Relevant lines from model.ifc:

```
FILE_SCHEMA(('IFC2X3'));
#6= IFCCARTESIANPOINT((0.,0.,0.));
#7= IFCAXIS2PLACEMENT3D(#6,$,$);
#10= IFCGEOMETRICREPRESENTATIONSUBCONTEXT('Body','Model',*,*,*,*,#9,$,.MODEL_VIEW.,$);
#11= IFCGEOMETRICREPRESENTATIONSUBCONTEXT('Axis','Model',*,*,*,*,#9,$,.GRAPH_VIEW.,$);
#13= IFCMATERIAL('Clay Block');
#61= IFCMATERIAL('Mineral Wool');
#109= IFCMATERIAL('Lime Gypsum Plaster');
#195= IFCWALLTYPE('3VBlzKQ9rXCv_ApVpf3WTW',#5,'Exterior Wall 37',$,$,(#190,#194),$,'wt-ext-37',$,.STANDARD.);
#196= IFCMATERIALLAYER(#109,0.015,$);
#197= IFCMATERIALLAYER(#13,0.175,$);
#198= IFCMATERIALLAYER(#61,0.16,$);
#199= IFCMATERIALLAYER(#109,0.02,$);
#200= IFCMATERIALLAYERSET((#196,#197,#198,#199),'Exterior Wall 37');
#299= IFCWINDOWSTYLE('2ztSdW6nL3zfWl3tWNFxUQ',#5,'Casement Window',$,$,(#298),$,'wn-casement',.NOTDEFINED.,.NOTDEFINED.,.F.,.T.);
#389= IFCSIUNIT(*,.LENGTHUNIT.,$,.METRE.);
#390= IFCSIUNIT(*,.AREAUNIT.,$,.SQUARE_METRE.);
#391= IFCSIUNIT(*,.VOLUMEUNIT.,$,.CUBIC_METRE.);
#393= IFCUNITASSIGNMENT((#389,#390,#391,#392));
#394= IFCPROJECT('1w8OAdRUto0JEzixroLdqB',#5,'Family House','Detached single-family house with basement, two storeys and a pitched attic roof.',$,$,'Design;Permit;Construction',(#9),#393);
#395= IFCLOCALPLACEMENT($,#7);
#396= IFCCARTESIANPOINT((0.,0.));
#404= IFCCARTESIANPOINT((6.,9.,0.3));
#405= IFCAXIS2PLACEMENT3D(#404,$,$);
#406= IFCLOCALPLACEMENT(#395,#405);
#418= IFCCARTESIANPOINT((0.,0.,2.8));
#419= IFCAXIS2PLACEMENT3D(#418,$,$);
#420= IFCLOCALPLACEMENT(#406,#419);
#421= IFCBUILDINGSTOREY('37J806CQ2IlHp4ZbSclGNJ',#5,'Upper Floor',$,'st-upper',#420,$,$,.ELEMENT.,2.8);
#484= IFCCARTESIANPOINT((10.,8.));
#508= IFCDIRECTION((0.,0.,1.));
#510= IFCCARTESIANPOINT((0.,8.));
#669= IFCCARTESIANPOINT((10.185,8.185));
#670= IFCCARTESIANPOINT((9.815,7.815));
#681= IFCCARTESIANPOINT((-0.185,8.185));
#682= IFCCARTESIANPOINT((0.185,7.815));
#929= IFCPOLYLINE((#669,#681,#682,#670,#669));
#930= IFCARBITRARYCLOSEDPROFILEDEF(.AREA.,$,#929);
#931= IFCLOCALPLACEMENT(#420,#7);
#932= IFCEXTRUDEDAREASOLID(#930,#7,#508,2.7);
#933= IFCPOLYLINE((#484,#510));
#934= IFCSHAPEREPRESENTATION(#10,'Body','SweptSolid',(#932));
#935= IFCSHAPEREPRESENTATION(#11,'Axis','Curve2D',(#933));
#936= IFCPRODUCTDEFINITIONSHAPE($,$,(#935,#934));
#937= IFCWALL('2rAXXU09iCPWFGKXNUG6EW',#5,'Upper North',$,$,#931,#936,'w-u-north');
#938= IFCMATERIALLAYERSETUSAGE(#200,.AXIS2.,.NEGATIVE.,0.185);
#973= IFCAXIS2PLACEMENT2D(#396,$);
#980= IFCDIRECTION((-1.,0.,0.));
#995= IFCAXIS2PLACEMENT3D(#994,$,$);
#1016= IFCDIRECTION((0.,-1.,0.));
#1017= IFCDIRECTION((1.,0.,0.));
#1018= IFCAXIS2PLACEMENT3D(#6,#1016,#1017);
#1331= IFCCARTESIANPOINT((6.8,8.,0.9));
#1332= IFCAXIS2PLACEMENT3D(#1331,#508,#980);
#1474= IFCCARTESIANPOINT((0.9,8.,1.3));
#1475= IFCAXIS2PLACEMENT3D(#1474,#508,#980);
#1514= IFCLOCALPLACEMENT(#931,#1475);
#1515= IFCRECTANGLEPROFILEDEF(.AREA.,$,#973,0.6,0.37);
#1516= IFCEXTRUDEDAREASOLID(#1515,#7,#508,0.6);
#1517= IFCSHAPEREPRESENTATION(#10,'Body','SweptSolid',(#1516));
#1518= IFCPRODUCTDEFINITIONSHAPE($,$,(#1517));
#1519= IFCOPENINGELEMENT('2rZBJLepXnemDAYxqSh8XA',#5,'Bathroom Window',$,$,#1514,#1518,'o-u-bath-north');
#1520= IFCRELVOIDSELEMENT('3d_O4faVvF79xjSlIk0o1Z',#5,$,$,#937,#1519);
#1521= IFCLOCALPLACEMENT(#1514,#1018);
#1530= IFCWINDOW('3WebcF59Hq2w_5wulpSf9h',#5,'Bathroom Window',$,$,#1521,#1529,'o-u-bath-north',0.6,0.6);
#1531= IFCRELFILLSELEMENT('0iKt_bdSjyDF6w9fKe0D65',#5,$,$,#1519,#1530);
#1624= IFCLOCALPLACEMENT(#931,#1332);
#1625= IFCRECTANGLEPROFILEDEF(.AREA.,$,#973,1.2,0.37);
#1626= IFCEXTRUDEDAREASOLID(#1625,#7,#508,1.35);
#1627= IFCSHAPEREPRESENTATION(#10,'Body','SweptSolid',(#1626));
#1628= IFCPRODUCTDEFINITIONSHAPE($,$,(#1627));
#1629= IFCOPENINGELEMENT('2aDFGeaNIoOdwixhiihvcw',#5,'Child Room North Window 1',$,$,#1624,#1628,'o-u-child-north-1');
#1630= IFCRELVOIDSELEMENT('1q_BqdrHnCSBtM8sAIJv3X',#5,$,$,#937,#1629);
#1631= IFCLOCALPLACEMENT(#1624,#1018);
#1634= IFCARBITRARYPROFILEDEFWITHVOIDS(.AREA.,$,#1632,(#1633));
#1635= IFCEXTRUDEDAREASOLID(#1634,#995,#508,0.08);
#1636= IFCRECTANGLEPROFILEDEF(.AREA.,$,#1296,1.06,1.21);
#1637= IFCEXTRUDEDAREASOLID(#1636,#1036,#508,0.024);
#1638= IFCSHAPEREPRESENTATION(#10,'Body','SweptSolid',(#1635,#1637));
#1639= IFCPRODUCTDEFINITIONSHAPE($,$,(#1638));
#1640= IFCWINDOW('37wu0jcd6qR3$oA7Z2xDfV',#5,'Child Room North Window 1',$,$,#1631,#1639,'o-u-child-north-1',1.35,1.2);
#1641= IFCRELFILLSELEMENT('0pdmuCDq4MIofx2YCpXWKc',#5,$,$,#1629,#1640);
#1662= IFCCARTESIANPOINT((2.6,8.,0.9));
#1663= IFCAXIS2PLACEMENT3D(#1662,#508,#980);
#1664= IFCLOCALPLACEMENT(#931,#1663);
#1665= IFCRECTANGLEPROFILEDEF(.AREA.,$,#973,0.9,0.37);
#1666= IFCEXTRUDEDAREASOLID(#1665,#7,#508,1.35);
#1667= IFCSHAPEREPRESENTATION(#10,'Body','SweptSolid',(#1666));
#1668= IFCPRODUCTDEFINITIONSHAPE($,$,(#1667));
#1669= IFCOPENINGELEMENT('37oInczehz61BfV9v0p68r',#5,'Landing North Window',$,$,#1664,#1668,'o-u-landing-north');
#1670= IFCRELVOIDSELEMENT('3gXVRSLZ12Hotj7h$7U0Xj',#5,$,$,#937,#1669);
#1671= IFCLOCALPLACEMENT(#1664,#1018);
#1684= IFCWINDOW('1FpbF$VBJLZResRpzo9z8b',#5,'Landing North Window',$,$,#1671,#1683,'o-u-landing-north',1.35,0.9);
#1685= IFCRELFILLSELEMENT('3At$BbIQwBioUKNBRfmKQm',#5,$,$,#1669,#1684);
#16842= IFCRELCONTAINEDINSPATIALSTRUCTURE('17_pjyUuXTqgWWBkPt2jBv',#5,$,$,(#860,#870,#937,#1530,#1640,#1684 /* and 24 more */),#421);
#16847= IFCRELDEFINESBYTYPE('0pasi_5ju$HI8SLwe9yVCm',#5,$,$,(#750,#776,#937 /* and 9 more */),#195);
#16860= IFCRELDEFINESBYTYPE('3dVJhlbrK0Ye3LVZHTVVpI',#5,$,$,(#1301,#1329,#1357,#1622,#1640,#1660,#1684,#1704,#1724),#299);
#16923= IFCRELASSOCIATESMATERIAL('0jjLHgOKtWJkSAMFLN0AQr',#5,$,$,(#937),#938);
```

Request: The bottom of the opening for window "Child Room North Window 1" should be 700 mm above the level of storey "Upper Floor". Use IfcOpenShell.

```python
import numpy as np
import ifcopenshell
import ifcopenshell.api.geometry
import ifcopenshell.geom
import ifcopenshell.util.element
import ifcopenshell.util.placement
import ifcopenshell.util.shape
import ifcopenshell.util.unit

model = ifcopenshell.open("model.ifc")
unit_scale = ifcopenshell.util.unit.calculate_unit_scale(model)

window = model.by_id(1640)
opening = window.FillsVoids[0].RelatingOpeningElement
storey = ifcopenshell.util.element.get_container(window, ifc_class="IfcBuildingStorey")
level = ifcopenshell.util.placement.get_local_placement(storey.ObjectPlacement)[2, 3]

# The opening's origin need not be at the sill, so measure its lowest point.
shape = ifcopenshell.geom.create_shape(ifcopenshell.geom.settings(), opening)
bottom = ifcopenshell.util.shape.get_shape_bottom_elevation(shape, shape.geometry) / unit_scale
dz = level + 0.7 - bottom

shift = np.array([0.0, 0.0, dz])
# The window is placed relative to its opening, so it follows when the opening moves.
matrix = ifcopenshell.util.placement.get_local_placement(opening.ObjectPlacement)
matrix[:3, 3] += shift
ifcopenshell.api.geometry.edit_object_placement(
    model, product=opening, matrix=matrix, is_si=False, should_transform_children=True
)

print(f"moved by {dz * unit_scale:+.3f} m")

model.write("model_v2.ifc")
```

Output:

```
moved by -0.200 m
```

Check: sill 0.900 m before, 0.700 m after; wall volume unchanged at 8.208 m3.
